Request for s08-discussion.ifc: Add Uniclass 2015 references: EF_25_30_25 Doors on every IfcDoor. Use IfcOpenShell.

First a look at what the model holds.

```python
import ifcopenshell

model = ifcopenshell.open("s08-discussion.ifc")
print(model.schema)
print("classifications:", [c.Name for c in model.by_type("IfcClassification")])
for ifc_class in ("IfcDoor", "IfcRoof", "IfcStair", "IfcWall", "IfcWindow"):
    print(ifc_class, len(model.by_type(ifc_class)))
```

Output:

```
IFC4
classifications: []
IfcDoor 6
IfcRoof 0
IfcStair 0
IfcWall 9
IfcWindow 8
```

```python
import ifcopenshell
import ifcopenshell.api.classification

model = ifcopenshell.open("s08-discussion.ifc")

system = ifcopenshell.api.classification.add_classification(model, classification="Uniclass 2015")

codes = {
    "IfcDoor": ("EF_25_30_25", "Doors"),
}
for ifc_class, (code, name) in codes.items():
    products = model.by_type(ifc_class)
    ifcopenshell.api.classification.add_reference(
        model, products=products, classification=system, identification=code, name=name
    )
    print(code, len(products))

model.write("s08-discussion_edited.ifc")
```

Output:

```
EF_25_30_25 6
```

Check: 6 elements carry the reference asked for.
